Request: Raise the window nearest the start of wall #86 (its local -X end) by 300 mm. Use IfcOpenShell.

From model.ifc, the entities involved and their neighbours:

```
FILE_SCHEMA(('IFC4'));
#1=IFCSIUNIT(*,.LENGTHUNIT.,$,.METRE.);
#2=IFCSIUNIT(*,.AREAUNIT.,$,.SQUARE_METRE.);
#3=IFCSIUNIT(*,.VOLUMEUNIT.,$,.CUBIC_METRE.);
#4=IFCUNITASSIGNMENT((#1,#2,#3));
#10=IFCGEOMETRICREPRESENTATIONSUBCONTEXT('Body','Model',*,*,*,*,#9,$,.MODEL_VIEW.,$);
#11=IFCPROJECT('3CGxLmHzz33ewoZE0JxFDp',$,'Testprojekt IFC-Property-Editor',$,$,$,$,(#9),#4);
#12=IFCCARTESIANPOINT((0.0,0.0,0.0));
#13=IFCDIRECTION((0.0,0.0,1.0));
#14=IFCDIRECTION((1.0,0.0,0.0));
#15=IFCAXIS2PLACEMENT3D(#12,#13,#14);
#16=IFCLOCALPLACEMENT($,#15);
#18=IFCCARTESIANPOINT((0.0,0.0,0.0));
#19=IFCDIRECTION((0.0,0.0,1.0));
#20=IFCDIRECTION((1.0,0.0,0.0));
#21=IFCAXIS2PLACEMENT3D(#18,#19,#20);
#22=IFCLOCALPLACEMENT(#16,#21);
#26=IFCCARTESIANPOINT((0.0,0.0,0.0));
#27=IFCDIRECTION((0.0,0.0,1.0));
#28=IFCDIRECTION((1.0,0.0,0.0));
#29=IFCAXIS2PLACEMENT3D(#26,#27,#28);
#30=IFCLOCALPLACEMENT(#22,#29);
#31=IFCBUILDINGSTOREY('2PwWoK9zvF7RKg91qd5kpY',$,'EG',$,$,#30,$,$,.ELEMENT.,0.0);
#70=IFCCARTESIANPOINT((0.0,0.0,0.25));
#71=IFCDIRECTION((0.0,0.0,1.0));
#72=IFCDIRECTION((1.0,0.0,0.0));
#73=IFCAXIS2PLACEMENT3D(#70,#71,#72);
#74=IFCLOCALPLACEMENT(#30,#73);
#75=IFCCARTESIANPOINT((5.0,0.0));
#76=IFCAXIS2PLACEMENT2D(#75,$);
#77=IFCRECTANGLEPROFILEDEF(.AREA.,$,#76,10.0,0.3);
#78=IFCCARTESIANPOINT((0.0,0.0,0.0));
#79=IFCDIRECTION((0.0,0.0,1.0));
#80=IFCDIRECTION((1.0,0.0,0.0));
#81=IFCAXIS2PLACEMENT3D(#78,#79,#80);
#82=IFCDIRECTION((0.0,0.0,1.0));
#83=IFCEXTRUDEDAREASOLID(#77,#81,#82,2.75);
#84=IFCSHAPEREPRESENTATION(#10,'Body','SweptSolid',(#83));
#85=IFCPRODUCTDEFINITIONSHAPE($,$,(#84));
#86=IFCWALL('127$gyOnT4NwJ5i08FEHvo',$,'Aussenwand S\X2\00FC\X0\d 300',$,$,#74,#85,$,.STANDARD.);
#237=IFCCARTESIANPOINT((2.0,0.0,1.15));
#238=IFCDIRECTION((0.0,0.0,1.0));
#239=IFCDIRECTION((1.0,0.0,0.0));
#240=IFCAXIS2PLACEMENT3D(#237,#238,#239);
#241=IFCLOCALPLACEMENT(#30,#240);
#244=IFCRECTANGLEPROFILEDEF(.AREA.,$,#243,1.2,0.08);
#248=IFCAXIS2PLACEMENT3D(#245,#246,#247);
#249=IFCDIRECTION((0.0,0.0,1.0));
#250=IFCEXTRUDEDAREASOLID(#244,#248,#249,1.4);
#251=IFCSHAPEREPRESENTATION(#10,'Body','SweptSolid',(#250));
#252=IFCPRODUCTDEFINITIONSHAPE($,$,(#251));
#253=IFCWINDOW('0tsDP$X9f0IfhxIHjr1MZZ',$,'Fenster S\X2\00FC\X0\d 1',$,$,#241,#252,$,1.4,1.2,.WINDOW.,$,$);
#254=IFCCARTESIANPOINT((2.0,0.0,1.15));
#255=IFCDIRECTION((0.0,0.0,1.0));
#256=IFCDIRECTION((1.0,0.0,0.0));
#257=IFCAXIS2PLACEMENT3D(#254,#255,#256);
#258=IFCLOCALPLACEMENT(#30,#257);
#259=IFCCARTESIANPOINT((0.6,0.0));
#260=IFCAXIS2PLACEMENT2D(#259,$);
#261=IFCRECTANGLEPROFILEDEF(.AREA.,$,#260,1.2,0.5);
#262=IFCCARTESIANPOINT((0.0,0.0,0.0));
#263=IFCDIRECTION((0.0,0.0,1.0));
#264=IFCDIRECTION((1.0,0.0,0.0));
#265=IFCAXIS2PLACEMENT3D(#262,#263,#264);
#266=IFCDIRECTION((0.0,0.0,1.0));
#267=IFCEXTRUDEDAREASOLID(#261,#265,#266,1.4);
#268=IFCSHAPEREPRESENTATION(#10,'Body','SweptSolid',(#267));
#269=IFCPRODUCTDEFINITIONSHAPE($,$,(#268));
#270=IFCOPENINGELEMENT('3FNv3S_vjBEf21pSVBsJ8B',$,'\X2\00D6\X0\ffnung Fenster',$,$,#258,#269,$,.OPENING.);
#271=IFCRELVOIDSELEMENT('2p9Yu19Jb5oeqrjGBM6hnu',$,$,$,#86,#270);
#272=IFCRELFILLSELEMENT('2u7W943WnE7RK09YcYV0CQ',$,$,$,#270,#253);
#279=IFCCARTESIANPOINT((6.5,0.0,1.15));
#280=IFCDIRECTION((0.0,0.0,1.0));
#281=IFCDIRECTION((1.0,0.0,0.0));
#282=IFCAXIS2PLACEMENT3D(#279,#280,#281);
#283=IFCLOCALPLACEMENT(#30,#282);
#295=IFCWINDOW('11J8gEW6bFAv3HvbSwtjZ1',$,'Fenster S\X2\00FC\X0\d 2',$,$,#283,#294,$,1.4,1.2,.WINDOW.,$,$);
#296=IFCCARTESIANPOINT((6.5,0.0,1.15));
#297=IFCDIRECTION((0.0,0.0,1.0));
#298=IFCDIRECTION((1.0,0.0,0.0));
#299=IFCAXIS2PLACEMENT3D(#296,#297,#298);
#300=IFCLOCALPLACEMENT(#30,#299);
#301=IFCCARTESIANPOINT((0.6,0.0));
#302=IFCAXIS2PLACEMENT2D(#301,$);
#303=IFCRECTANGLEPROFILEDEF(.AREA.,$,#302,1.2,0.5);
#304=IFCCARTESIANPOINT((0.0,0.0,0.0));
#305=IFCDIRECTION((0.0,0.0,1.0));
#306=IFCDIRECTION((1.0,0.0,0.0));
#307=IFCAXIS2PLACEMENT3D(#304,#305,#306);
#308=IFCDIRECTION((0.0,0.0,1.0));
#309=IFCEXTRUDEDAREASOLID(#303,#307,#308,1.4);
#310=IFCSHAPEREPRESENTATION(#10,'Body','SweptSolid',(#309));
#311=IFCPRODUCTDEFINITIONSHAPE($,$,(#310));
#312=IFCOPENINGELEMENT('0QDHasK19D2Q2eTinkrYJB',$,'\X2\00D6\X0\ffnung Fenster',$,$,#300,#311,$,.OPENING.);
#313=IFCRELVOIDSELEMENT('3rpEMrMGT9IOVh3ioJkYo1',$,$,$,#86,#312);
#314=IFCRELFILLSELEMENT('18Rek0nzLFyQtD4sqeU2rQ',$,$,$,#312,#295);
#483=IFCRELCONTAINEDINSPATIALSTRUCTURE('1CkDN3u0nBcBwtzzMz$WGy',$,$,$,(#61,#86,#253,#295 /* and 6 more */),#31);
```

```python
import numpy as np
import ifcopenshell
import ifcopenshell.api.geometry
import ifcopenshell.util.placement
import ifcopenshell.util.unit

model = ifcopenshell.open("model.ifc")
unit_scale = ifcopenshell.util.unit.calculate_unit_scale(model)

window = model.by_id(253)
opening = window.FillsVoids[0].RelatingOpeningElement
dz = 0.3

shift = np.array([0.0, 0.0, dz])
# The window is not placed relative to its opening, so move both.
for product in (opening, window):
    matrix = ifcopenshell.util.placement.get_local_placement(product.ObjectPlacement)
    matrix[:3, 3] += shift
    ifcopenshell.api.geometry.edit_object_placement(model, product=product, matrix=matrix, is_si=False)

print(f"moved by {dz * unit_scale:+.3f} m")

model.write("model-out.ifc")
```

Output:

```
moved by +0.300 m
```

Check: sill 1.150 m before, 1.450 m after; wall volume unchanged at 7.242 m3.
